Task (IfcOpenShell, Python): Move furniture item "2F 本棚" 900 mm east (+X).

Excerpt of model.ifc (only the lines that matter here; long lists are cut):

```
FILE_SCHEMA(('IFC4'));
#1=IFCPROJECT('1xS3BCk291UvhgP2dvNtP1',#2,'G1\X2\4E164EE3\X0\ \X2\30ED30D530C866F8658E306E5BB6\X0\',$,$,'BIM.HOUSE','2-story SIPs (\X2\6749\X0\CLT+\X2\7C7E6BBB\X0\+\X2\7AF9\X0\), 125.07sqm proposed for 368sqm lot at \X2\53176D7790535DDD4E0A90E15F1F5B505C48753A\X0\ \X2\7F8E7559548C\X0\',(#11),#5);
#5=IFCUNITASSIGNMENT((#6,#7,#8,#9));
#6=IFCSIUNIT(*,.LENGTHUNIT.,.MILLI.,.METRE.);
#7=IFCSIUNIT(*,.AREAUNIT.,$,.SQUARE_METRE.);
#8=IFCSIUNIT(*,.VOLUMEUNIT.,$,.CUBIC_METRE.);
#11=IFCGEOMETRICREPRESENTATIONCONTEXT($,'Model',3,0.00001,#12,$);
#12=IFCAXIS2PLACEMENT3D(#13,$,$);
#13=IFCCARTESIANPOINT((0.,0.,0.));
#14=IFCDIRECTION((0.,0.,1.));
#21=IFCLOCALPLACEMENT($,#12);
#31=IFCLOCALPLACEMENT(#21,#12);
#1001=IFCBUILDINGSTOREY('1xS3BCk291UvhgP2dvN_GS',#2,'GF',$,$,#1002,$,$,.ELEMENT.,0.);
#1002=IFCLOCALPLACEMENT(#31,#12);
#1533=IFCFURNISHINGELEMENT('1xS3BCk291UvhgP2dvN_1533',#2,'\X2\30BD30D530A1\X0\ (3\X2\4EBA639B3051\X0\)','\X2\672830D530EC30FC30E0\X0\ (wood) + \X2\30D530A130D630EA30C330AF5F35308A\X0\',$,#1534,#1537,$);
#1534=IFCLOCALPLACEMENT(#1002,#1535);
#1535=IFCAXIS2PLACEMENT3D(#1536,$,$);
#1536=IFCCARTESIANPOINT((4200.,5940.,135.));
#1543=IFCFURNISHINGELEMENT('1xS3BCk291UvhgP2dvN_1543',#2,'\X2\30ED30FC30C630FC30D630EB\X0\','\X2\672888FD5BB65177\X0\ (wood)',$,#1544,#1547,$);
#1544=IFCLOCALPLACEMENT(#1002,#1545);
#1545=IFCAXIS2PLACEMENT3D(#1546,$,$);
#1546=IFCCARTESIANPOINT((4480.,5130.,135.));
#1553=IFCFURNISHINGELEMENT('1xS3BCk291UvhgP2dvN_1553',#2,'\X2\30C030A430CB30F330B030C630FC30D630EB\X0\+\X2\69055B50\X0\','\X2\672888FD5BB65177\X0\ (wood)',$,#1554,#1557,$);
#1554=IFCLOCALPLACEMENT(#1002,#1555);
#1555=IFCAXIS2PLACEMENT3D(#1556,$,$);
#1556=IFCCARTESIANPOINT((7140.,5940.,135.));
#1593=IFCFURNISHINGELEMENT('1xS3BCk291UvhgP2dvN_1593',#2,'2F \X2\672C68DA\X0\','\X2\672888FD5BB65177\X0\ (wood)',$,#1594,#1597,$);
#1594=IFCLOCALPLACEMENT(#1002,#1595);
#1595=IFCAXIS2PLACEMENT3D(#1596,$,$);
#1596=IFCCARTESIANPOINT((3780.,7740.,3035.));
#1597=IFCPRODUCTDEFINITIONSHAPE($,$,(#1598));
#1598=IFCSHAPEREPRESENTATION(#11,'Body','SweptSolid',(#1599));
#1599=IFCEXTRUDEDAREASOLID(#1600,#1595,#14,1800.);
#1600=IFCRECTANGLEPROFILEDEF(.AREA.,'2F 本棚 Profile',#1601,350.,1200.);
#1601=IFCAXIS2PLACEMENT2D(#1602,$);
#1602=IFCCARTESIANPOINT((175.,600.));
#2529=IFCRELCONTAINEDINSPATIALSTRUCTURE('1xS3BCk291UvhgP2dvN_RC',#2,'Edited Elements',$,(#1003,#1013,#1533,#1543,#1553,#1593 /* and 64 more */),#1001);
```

```python
import ifcopenshell
import ifcopenshell.api.geometry
import ifcopenshell.util.placement

model = ifcopenshell.open("model.ifc")

item = model.by_guid("1xS3BCk291UvhgP2dvN_1593")
matrix = ifcopenshell.util.placement.get_local_placement(item.ObjectPlacement)
matrix[0, 3] += 900.0
ifcopenshell.api.geometry.edit_object_placement(model, product=item, matrix=matrix, is_si=False)

print(ifcopenshell.util.placement.get_local_placement(item.ObjectPlacement).round(3) + 0.0)

model.write("model_updated.ifc")
```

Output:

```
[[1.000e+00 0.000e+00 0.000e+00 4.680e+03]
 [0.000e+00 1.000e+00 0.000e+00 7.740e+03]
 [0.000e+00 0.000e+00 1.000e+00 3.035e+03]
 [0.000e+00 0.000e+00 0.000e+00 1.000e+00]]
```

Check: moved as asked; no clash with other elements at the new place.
